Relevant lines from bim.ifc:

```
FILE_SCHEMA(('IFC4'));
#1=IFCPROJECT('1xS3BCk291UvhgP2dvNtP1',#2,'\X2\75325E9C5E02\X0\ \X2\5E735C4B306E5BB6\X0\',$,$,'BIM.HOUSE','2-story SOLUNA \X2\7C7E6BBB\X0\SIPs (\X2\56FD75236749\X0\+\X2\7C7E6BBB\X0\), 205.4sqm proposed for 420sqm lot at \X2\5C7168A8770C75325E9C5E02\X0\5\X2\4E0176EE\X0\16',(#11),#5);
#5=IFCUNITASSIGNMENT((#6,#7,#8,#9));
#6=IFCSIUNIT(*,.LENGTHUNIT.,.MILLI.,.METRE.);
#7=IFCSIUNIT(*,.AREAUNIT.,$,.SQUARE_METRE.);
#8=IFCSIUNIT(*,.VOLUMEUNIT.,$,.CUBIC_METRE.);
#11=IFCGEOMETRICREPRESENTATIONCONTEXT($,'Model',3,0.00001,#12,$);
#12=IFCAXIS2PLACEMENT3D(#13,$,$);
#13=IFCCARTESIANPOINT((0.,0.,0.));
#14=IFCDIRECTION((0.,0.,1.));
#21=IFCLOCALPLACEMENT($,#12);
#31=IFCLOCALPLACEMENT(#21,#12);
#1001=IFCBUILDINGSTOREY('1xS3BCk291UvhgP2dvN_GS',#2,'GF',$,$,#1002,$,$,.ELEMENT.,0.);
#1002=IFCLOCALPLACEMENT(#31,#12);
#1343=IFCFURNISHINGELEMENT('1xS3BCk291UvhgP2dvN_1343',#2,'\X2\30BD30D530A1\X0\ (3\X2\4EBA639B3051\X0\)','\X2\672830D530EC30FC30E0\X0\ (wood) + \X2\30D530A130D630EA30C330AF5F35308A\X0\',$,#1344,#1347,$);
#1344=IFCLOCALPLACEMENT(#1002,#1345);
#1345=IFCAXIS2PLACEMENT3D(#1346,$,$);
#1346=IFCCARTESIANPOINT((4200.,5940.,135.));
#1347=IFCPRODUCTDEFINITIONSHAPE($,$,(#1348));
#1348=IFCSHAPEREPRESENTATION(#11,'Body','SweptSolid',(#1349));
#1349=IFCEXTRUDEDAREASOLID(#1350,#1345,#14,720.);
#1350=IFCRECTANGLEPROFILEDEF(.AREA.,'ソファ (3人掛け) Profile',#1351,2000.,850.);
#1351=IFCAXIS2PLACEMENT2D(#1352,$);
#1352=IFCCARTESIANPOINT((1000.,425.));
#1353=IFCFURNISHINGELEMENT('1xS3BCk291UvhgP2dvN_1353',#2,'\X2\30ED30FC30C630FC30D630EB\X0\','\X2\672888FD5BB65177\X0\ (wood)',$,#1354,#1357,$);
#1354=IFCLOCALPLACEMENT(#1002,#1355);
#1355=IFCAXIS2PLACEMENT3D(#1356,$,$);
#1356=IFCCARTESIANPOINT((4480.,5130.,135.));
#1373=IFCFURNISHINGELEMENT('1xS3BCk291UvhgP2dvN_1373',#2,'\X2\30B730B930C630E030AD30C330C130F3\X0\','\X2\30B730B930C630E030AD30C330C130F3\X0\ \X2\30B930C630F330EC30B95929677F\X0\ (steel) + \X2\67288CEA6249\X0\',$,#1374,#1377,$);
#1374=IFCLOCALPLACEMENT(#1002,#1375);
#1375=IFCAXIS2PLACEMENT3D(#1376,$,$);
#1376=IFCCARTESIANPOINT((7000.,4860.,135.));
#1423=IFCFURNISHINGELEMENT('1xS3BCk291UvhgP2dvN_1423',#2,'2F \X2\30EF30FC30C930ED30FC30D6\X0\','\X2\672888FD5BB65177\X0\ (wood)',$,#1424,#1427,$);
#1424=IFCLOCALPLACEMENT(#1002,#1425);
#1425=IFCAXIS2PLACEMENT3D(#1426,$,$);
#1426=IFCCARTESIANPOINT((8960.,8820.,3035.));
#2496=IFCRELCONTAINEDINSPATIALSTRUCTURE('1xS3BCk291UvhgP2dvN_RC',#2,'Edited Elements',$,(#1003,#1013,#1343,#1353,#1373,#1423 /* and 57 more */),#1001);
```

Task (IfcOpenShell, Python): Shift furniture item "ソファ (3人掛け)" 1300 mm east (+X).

```python
import ifcopenshell
import ifcopenshell.api.geometry
import ifcopenshell.util.placement
import ifcopenshell.util.unit

model = ifcopenshell.open("bim.ifc")
unit_scale = ifcopenshell.util.unit.calculate_unit_scale(model)

item = model.by_guid("1xS3BCk291UvhgP2dvN_1343")
matrix = ifcopenshell.util.placement.get_local_placement(item.ObjectPlacement)
matrix[0, 3] += 1.3 / unit_scale
ifcopenshell.api.geometry.edit_object_placement(model, product=item, matrix=matrix, is_si=False)

print(ifcopenshell.util.placement.get_local_placement(item.ObjectPlacement).round(3) + 0.0)

model.write("bim_rev.ifc")
```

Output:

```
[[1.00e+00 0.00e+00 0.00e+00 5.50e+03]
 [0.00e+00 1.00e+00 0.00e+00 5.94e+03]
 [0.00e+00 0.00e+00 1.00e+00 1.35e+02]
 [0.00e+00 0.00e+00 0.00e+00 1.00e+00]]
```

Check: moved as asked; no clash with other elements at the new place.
